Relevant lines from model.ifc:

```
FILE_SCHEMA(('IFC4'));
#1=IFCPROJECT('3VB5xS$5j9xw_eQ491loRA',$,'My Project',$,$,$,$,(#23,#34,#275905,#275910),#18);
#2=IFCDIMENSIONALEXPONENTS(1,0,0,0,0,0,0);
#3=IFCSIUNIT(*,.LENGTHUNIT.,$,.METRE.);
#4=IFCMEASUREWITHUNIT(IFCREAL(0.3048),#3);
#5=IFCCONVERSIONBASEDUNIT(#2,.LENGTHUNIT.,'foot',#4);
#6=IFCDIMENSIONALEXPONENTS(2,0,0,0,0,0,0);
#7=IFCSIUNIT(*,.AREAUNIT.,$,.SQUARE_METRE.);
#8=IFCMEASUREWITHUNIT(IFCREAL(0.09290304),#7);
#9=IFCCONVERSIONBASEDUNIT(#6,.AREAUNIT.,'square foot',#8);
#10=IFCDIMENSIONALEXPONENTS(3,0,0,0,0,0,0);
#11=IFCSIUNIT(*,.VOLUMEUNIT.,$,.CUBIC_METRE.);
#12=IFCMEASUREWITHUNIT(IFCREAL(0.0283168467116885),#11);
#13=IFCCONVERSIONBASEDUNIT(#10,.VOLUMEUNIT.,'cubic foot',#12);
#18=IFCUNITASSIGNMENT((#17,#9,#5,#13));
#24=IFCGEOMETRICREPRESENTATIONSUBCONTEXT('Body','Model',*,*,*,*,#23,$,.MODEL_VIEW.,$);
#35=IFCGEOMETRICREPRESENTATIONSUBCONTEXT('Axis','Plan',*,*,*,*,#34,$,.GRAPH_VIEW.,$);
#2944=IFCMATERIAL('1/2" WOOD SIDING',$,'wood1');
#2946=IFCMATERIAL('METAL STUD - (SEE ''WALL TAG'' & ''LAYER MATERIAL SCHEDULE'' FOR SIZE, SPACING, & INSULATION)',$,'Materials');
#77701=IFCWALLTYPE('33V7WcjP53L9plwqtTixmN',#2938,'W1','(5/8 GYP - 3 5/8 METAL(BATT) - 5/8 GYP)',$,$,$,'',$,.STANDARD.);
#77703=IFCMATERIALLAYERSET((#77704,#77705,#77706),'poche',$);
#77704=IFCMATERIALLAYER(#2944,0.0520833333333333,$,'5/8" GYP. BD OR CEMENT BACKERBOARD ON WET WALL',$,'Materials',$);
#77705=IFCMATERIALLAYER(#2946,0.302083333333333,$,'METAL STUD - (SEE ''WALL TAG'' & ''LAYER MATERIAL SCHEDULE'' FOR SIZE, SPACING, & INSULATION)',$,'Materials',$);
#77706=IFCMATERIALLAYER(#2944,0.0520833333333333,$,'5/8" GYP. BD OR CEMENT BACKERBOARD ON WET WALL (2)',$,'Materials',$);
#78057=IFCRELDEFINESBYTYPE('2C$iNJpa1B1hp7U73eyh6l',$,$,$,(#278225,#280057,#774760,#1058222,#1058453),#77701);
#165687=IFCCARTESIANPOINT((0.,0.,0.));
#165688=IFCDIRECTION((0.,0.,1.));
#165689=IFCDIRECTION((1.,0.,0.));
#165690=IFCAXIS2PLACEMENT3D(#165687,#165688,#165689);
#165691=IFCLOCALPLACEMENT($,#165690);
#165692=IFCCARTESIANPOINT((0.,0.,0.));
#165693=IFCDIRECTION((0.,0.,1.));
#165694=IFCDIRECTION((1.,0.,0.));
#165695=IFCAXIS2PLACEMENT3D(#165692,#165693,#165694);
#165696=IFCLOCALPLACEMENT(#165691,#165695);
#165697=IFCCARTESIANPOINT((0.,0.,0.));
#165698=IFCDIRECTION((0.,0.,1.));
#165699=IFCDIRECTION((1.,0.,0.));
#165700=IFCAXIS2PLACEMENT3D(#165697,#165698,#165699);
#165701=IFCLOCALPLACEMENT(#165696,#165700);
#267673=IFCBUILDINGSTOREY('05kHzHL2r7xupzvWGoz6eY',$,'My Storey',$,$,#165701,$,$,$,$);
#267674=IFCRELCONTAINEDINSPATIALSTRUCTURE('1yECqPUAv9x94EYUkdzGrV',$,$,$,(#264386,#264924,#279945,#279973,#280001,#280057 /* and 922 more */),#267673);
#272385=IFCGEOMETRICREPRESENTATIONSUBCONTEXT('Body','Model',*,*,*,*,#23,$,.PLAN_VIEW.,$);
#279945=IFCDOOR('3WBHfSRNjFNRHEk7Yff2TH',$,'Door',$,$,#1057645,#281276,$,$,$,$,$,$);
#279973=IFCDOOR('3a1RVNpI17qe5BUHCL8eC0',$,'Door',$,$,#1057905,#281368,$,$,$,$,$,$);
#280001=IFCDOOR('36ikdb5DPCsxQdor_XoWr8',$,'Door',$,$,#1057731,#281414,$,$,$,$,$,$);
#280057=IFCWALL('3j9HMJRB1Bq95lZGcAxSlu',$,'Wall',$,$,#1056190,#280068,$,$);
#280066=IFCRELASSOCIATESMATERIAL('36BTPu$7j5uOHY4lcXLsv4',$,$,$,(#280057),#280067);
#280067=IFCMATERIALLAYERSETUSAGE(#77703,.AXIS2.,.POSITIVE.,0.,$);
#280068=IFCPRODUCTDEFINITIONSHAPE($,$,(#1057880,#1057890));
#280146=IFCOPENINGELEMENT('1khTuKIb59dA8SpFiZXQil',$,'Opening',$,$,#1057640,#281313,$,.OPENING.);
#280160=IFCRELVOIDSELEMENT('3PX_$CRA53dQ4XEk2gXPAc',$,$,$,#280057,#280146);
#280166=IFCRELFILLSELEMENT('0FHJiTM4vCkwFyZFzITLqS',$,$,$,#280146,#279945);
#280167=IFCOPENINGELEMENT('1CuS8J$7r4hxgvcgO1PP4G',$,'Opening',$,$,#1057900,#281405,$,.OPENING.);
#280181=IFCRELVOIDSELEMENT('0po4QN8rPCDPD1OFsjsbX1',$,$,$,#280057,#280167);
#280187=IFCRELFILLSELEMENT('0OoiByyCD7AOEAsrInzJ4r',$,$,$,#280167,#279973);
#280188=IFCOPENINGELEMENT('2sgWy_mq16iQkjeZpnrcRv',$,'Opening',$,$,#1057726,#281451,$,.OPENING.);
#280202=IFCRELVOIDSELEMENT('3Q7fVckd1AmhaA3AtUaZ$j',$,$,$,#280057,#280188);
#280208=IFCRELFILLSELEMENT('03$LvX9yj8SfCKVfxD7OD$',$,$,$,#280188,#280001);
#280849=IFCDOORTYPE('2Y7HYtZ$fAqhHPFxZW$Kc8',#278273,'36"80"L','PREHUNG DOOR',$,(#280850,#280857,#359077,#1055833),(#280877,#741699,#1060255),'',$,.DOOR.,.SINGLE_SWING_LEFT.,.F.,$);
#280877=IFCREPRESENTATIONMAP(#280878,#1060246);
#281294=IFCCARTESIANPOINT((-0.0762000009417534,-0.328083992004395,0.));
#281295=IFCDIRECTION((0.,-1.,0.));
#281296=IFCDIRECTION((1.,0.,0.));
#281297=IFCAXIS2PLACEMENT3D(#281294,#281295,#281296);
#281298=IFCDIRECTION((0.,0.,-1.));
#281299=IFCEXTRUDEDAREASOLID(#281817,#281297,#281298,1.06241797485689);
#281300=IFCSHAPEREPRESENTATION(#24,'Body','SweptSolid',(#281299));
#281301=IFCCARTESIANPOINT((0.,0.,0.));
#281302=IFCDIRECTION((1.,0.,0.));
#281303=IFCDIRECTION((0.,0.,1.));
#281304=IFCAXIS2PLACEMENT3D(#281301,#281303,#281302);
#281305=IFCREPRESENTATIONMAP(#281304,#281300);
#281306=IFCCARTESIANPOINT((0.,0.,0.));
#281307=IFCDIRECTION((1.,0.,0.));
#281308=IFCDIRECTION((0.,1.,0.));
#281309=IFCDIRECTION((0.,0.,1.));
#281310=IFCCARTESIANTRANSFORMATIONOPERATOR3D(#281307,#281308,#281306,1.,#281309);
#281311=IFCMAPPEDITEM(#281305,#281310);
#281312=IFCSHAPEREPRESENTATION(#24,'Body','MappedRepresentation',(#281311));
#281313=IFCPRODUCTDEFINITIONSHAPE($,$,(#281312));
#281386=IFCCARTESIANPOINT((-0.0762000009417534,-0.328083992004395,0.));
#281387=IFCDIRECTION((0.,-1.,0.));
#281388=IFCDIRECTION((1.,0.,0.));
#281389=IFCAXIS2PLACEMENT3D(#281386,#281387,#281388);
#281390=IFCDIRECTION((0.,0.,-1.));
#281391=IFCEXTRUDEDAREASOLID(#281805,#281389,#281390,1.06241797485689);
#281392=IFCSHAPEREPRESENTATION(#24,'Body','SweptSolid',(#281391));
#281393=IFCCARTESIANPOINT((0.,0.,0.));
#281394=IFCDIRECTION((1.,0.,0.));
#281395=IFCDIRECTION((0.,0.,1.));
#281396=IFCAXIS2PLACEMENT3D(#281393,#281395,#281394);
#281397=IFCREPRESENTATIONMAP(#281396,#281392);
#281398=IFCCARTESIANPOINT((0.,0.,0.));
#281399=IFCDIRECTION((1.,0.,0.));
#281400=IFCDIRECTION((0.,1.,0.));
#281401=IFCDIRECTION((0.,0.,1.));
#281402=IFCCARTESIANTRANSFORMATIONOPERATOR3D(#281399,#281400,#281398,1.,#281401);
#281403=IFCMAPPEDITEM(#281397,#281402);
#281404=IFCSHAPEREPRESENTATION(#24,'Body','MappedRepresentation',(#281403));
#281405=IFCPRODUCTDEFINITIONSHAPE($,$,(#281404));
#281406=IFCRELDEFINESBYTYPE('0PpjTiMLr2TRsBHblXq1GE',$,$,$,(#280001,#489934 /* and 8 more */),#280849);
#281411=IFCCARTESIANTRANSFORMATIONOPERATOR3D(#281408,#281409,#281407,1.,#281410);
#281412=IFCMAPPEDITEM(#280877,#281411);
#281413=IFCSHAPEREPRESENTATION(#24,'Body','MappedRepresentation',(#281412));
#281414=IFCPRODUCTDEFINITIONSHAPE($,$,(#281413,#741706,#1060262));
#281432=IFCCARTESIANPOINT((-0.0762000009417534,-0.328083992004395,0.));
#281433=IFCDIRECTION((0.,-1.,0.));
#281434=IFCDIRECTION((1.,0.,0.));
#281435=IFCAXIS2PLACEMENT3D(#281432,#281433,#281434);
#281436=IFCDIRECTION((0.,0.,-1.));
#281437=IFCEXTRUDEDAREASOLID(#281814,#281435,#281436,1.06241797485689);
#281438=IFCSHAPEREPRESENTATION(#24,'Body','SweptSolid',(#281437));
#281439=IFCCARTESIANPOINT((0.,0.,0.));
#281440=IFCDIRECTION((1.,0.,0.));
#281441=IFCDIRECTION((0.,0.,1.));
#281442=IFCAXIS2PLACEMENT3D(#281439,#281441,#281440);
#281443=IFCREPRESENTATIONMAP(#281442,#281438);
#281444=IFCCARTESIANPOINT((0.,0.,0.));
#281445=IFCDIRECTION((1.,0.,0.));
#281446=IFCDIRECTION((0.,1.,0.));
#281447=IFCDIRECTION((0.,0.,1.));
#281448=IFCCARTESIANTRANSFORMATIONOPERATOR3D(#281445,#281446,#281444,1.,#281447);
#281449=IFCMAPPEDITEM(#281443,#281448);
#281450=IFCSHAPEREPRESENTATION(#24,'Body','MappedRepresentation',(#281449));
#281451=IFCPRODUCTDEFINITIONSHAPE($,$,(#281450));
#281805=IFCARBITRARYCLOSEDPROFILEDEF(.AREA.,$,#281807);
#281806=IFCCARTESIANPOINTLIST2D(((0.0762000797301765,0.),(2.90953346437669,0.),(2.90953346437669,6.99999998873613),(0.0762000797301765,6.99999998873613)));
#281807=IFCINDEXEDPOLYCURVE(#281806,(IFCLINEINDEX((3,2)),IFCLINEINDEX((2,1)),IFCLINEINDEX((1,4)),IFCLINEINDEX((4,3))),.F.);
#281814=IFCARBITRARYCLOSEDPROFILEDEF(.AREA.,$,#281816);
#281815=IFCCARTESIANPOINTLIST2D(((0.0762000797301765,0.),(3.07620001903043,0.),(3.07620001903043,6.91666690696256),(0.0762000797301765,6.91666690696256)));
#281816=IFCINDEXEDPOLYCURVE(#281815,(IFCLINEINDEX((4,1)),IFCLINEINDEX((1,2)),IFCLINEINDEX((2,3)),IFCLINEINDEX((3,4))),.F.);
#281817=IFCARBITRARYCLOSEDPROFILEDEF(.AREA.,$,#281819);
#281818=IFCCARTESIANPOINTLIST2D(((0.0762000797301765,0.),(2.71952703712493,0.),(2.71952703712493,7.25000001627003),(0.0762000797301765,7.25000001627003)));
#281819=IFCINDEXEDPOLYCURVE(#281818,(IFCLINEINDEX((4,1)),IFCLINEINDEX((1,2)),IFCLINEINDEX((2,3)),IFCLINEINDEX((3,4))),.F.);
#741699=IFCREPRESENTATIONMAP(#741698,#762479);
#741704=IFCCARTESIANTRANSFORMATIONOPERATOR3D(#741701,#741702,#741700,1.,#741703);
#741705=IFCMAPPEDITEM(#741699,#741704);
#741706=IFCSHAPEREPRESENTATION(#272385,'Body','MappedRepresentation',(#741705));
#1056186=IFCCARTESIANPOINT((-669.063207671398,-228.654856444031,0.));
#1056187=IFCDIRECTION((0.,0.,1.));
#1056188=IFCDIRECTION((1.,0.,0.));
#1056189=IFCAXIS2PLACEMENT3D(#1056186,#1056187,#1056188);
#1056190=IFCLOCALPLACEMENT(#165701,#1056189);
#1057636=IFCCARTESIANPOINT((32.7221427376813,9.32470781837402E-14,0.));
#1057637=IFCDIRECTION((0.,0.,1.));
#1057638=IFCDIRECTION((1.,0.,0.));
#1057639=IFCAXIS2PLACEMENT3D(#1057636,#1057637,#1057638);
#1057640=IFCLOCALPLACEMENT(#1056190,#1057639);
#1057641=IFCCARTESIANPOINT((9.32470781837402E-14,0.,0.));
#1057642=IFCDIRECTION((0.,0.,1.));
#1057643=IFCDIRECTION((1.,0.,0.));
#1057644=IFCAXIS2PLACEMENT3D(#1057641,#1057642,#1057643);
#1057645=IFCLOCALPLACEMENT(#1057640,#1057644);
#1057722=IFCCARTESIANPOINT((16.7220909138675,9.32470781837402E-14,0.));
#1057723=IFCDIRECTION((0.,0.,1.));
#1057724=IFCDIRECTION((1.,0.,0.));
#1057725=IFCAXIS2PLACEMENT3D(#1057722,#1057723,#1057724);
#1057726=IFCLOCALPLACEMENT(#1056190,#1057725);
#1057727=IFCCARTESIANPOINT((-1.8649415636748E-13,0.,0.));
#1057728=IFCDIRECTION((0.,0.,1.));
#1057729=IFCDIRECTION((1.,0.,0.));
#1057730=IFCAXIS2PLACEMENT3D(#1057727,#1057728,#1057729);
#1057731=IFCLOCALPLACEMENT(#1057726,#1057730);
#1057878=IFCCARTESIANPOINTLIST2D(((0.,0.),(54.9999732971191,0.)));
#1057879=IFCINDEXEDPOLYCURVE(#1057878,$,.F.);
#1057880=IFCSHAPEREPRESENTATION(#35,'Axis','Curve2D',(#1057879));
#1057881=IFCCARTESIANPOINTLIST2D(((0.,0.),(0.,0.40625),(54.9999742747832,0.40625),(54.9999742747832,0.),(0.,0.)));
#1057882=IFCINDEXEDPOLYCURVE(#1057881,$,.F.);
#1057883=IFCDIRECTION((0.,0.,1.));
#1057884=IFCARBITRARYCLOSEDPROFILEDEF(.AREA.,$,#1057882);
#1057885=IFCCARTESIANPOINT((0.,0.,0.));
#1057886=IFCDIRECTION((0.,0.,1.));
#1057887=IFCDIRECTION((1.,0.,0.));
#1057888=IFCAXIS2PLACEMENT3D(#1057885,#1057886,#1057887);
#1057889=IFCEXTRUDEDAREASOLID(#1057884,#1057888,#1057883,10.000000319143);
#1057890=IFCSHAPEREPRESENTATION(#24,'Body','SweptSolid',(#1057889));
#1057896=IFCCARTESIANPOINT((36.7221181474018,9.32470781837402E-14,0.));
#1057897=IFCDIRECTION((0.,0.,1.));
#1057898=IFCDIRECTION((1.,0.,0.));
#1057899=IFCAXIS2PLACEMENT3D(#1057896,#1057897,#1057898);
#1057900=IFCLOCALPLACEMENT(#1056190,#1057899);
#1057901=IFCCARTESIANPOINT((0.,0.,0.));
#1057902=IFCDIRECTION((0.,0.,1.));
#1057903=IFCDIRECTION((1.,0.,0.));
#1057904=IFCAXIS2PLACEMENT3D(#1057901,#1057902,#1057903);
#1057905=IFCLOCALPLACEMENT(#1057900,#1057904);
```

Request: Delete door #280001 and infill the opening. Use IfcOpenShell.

```python
import ifcopenshell
import ifcopenshell.api.feature
import ifcopenshell.api.root
import ifcopenshell.geom
import ifcopenshell.util.shape

model = ifcopenshell.open("model.ifc")
settings = ifcopenshell.geom.settings()


def volume(element):
    """Net volume in cubic metres, openings subtracted."""
    shape = ifcopenshell.geom.create_shape(settings, element)
    return ifcopenshell.util.shape.get_volume(shape.geometry)


door = model.by_guid("36ikdb5DPCsxQdor_XoWr8")
opening = door.FillsVoids[0].RelatingOpeningElement
wall = opening.VoidsElements[0].RelatingBuildingElement
before = volume(wall)

ifcopenshell.api.root.remove_product(model, product=door)
ifcopenshell.api.feature.remove_feature(model, feature=opening)

after = volume(wall)

print(f"wall volume {before:.3f} -> {after:.3f} m3")

model.write("model_v2.ifc")
```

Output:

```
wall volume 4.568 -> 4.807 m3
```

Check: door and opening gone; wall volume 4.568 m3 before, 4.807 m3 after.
